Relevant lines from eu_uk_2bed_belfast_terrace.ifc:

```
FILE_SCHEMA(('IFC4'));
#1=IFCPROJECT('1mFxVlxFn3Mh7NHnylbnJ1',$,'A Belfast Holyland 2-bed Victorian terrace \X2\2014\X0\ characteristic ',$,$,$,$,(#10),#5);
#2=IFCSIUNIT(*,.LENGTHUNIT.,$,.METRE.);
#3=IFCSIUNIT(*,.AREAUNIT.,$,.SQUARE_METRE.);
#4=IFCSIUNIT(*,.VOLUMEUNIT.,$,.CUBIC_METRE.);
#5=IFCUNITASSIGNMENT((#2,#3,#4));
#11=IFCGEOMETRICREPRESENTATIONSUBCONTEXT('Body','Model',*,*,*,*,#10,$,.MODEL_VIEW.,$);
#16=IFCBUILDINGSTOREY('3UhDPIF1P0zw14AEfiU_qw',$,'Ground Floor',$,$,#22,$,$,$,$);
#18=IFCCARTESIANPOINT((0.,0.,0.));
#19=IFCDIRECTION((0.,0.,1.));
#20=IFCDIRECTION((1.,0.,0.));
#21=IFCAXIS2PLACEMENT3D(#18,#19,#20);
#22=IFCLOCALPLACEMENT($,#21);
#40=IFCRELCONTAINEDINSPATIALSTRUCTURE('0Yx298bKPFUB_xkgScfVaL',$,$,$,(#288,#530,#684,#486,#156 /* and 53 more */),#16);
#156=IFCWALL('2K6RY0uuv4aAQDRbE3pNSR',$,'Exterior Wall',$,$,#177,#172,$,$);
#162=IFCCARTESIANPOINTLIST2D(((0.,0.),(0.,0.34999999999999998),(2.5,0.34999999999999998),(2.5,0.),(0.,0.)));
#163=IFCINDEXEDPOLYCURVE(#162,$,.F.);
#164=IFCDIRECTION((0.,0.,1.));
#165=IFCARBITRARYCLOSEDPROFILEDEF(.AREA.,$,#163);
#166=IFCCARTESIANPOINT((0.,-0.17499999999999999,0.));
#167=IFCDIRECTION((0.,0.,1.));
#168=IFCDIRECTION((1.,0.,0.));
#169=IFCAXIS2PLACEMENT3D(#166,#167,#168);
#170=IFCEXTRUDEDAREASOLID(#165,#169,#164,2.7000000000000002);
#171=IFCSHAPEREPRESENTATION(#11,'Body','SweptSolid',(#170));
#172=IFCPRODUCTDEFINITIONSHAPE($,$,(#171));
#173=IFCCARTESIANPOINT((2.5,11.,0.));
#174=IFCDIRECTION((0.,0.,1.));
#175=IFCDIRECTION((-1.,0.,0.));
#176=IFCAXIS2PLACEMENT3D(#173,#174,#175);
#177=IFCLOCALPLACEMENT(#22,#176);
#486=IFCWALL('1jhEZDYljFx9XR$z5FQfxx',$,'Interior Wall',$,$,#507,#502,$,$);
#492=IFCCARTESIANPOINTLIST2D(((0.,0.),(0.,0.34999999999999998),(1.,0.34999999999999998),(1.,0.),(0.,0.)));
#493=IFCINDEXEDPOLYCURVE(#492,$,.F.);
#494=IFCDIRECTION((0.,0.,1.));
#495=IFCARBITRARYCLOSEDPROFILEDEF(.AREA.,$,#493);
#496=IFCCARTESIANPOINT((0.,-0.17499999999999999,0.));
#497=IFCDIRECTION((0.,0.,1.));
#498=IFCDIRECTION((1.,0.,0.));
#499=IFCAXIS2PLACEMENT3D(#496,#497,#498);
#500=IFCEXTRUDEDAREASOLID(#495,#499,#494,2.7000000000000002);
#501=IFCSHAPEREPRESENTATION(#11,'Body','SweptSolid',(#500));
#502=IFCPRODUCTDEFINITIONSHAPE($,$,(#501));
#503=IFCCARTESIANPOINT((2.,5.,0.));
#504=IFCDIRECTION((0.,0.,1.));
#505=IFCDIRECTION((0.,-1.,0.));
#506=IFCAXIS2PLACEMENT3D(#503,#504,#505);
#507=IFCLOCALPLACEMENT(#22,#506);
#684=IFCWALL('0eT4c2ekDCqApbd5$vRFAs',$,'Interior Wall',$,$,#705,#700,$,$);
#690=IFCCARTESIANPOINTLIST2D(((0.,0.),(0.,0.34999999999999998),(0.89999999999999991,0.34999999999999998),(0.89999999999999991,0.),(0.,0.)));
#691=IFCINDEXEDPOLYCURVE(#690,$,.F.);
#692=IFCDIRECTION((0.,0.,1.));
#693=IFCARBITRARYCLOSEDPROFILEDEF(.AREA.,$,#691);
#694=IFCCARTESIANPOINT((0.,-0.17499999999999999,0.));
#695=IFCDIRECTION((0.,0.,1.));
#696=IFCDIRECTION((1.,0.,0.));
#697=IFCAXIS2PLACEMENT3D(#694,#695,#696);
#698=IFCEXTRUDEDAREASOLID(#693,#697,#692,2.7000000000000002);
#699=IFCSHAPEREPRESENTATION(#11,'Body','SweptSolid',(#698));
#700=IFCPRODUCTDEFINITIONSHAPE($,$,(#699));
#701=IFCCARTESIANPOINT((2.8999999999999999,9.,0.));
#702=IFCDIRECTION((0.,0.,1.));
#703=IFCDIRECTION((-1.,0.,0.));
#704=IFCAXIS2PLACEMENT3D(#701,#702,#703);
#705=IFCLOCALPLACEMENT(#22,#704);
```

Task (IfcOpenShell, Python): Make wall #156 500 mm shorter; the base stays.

```python
import ifcopenshell
import ifcopenshell.geom
import ifcopenshell.util.representation
import ifcopenshell.util.shape

model = ifcopenshell.open("eu_uk_2bed_belfast_terrace.ifc")
settings = ifcopenshell.geom.settings()


def volume(element):
    """Net volume in cubic metres, openings subtracted."""
    shape = ifcopenshell.geom.create_shape(settings, element)
    return ifcopenshell.util.shape.get_volume(shape.geometry)


wall = model.by_guid("2K6RY0uuv4aAQDRbE3pNSR")
before = volume(wall)

body = ifcopenshell.util.representation.get_representation(wall, "Model", "Body")
solid = body.Items[0]
old_height = solid.Depth
solid.Depth -= 0.5
after = volume(wall)

print(f"height {old_height:g} -> {solid.Depth:g}, volume {before:.3f} -> {after:.3f} m3")

model.write("eu_uk_2bed_belfast_terrace_updated.ifc")
```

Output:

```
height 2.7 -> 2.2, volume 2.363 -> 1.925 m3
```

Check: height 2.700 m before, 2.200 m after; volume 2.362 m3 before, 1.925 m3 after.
